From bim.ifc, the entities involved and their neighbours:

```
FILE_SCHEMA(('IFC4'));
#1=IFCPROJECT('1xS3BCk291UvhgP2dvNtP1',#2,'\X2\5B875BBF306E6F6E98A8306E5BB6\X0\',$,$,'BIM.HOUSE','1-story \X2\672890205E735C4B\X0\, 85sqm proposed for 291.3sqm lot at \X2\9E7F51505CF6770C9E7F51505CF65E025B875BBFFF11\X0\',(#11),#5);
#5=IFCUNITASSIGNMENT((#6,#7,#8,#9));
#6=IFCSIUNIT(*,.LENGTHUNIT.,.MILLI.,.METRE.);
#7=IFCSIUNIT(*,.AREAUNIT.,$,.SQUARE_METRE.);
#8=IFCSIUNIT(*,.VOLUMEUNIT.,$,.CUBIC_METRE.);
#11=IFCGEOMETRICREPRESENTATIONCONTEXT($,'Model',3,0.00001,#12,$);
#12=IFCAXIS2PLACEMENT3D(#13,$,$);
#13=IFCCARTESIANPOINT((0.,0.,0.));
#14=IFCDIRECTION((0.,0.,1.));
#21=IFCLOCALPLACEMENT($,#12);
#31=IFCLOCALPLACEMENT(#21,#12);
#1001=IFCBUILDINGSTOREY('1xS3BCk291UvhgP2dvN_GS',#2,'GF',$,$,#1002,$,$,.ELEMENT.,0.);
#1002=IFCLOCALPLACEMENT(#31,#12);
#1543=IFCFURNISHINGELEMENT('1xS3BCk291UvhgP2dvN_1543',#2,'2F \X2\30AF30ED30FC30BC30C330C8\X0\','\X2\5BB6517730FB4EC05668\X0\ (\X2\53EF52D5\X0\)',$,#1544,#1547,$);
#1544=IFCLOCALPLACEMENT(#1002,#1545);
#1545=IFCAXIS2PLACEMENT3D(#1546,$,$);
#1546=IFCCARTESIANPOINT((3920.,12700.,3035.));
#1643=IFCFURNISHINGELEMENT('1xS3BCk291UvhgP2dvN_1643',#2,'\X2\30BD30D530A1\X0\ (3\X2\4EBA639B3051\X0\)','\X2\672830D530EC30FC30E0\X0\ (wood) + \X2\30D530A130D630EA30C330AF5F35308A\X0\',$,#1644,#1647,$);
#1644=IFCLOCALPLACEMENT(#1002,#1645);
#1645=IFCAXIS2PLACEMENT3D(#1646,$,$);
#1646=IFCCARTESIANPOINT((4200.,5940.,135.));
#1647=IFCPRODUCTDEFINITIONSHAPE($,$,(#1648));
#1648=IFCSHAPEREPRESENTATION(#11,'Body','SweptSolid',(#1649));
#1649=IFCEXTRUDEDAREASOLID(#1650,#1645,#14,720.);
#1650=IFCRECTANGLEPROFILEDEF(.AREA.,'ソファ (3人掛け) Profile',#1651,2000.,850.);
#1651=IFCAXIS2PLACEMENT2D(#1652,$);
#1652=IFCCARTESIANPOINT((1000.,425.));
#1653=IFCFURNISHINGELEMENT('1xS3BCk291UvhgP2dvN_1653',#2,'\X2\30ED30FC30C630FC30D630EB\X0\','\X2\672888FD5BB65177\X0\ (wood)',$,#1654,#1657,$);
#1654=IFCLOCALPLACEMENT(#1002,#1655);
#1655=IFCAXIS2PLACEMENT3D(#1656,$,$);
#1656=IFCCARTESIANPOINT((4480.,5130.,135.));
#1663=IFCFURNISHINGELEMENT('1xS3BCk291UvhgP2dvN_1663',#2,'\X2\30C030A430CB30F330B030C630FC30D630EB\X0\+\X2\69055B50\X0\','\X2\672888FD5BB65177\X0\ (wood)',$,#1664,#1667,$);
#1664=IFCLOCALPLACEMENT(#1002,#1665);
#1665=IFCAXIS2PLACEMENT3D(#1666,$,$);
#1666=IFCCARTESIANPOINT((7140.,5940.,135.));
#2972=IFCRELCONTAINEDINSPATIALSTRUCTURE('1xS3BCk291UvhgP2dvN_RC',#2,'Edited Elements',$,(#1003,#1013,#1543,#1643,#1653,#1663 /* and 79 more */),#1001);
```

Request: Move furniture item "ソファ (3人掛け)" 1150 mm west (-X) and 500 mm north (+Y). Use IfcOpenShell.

```python
import ifcopenshell
import ifcopenshell.api.geometry
import ifcopenshell.util.placement
import ifcopenshell.util.unit

model = ifcopenshell.open("bim.ifc")
unit_scale = ifcopenshell.util.unit.calculate_unit_scale(model)

item = model.by_guid("1xS3BCk291UvhgP2dvN_1643")
matrix = ifcopenshell.util.placement.get_local_placement(item.ObjectPlacement)
matrix[0, 3] -= 1.15 / unit_scale
matrix[1, 3] += 0.5 / unit_scale
ifcopenshell.api.geometry.edit_object_placement(model, product=item, matrix=matrix, is_si=False)

print(ifcopenshell.util.placement.get_local_placement(item.ObjectPlacement).round(3) + 0.0)

model.write("bim_edited.ifc")
```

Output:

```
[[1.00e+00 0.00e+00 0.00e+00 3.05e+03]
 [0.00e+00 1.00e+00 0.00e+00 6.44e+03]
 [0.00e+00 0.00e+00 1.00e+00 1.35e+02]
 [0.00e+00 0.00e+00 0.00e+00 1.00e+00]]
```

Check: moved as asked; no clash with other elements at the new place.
